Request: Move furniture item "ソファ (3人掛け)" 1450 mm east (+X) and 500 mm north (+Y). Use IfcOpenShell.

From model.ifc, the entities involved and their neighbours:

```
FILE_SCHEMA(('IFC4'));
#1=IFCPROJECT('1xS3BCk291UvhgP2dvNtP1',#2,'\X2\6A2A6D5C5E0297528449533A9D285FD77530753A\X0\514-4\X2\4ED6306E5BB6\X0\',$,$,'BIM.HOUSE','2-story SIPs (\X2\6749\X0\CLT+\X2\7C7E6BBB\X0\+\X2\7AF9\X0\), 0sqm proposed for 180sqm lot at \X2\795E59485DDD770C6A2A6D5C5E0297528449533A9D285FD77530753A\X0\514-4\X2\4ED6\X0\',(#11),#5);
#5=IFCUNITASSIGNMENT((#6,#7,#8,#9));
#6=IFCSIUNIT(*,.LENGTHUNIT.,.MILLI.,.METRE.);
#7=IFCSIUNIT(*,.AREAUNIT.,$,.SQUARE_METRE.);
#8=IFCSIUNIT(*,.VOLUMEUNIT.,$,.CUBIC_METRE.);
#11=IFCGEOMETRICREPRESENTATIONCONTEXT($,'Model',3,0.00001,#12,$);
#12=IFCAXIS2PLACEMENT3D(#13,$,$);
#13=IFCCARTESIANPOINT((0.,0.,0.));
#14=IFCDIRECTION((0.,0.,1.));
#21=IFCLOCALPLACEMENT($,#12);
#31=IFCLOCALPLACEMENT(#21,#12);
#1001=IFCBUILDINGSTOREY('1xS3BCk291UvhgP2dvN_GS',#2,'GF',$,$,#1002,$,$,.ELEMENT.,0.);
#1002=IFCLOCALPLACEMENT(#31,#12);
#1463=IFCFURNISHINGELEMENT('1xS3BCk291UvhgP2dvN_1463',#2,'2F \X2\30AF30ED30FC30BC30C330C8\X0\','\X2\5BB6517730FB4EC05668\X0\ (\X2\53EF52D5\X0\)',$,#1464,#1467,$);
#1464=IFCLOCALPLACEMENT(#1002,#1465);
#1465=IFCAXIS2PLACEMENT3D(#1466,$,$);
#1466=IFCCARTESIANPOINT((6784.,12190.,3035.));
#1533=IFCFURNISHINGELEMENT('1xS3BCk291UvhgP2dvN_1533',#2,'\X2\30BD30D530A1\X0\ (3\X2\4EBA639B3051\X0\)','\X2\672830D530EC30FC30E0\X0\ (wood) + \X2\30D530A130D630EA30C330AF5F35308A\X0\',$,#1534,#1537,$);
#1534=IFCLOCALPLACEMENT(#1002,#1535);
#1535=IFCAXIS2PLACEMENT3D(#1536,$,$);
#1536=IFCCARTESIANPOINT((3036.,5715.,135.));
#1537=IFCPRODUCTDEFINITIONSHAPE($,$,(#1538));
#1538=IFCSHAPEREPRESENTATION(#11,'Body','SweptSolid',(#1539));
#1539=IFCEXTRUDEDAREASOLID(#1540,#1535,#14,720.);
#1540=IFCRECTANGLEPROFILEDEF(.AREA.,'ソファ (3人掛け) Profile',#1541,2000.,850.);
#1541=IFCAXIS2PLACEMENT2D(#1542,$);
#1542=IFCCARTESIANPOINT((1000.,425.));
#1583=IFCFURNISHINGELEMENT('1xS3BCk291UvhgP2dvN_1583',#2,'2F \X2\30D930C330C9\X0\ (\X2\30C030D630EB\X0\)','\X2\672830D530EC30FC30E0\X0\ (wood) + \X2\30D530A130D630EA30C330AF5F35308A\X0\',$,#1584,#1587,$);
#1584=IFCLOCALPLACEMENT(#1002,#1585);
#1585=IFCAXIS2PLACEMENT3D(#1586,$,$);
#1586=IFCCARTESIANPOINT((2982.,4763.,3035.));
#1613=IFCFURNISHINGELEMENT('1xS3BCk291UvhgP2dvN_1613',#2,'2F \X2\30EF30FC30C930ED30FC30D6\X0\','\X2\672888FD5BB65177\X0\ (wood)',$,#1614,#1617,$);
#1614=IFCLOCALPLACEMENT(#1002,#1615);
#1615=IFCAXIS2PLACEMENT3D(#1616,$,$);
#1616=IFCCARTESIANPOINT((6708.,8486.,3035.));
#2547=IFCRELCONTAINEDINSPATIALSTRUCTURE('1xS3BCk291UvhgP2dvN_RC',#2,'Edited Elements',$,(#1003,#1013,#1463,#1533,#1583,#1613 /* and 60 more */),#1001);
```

```python
import ifcopenshell
import ifcopenshell.api.geometry
import ifcopenshell.util.placement
import ifcopenshell.util.unit

model = ifcopenshell.open("model.ifc")
unit_scale = ifcopenshell.util.unit.calculate_unit_scale(model)

item = model.by_id(1533)
matrix = ifcopenshell.util.placement.get_local_placement(item.ObjectPlacement)
matrix[0, 3] += 1.45 / unit_scale
matrix[1, 3] += 0.5 / unit_scale
ifcopenshell.api.geometry.edit_object_placement(model, product=item, matrix=matrix, is_si=False)

print(ifcopenshell.util.placement.get_local_placement(item.ObjectPlacement).round(3) + 0.0)

model.write("model-out.ifc")
```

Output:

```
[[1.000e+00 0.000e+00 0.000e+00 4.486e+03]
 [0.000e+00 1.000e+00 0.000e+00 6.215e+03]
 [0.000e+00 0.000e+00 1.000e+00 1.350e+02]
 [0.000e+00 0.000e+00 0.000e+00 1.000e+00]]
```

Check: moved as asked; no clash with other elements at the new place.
